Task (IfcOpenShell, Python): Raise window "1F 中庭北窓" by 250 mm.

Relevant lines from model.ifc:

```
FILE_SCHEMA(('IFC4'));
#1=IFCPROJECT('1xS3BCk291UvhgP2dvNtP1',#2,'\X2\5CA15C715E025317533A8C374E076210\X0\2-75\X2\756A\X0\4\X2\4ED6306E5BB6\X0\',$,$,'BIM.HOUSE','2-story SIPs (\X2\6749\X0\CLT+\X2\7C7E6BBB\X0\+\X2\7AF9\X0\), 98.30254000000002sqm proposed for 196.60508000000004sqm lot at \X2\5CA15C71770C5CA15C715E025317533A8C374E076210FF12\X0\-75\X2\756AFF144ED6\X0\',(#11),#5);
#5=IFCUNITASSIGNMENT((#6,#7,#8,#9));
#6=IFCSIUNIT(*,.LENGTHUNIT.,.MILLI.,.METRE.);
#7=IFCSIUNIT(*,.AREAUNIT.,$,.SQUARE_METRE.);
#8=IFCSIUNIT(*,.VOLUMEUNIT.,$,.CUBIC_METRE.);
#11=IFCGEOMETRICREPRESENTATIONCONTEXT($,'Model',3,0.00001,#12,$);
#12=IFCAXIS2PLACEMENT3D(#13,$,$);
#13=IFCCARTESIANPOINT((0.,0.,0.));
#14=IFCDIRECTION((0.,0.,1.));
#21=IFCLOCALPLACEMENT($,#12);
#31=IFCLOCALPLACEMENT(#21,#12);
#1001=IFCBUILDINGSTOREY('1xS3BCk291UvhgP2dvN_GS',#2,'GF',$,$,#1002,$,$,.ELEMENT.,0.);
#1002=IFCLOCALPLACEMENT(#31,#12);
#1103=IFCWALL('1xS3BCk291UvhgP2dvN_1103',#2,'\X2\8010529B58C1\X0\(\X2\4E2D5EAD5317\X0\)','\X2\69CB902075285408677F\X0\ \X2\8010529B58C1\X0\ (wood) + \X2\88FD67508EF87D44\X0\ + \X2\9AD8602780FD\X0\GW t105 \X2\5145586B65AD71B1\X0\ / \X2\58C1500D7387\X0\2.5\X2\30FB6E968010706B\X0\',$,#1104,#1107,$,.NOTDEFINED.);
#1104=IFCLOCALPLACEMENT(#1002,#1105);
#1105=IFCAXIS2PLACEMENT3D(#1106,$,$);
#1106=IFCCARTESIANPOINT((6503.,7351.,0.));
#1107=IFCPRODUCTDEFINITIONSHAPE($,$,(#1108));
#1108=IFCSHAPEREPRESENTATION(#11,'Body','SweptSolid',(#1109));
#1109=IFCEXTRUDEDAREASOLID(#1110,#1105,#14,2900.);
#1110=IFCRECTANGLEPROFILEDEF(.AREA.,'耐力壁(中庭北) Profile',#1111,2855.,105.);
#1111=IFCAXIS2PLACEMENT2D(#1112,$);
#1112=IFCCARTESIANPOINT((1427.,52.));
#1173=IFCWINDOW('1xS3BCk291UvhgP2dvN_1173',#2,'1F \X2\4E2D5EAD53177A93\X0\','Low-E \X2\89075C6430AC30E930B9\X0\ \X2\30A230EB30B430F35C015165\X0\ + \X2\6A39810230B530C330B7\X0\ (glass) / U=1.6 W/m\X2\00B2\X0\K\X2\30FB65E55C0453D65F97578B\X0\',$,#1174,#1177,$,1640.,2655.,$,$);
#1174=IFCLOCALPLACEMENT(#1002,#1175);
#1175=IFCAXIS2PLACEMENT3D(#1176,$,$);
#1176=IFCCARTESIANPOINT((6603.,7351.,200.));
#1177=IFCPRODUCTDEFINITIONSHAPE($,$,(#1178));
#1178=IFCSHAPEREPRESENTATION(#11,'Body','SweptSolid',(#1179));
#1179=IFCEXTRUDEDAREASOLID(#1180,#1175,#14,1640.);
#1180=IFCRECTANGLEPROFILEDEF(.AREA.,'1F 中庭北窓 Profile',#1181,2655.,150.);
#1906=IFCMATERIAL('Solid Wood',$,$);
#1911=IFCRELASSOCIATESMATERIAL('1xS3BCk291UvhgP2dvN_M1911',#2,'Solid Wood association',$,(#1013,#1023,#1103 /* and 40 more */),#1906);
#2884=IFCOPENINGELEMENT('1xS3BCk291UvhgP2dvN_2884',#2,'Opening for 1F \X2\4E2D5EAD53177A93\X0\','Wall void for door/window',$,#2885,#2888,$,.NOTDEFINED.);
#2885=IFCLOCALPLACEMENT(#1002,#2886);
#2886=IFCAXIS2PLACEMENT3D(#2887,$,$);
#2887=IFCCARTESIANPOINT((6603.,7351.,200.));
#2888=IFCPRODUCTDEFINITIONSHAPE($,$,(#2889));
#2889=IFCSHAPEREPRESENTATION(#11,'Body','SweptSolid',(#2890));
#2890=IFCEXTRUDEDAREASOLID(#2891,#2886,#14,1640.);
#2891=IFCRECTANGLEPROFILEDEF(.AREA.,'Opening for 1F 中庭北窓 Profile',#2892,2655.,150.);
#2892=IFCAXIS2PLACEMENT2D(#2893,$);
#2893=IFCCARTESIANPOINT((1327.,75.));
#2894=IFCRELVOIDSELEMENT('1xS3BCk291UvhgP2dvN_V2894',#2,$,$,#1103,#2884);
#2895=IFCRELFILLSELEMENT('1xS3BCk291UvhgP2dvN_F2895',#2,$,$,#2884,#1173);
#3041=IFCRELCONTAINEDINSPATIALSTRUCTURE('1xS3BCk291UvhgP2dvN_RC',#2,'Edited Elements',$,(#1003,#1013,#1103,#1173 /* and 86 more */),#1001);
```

```python
import numpy as np
import ifcopenshell
import ifcopenshell.api.geometry
import ifcopenshell.util.placement
import ifcopenshell.util.unit

model = ifcopenshell.open("model.ifc")
unit_scale = ifcopenshell.util.unit.calculate_unit_scale(model)

window = model.by_guid("1xS3BCk291UvhgP2dvN_1173")
opening = window.FillsVoids[0].RelatingOpeningElement
dz = 250.0

shift = np.array([0.0, 0.0, dz])
# The window is not placed relative to its opening, so move both.
for product in (opening, window):
    matrix = ifcopenshell.util.placement.get_local_placement(product.ObjectPlacement)
    matrix[:3, 3] += shift
    ifcopenshell.api.geometry.edit_object_placement(model, product=product, matrix=matrix, is_si=False)

print(f"moved by {dz * unit_scale:+.3f} m")

model.write("model_edited.ifc")
```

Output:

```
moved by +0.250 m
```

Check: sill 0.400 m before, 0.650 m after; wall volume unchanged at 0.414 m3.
